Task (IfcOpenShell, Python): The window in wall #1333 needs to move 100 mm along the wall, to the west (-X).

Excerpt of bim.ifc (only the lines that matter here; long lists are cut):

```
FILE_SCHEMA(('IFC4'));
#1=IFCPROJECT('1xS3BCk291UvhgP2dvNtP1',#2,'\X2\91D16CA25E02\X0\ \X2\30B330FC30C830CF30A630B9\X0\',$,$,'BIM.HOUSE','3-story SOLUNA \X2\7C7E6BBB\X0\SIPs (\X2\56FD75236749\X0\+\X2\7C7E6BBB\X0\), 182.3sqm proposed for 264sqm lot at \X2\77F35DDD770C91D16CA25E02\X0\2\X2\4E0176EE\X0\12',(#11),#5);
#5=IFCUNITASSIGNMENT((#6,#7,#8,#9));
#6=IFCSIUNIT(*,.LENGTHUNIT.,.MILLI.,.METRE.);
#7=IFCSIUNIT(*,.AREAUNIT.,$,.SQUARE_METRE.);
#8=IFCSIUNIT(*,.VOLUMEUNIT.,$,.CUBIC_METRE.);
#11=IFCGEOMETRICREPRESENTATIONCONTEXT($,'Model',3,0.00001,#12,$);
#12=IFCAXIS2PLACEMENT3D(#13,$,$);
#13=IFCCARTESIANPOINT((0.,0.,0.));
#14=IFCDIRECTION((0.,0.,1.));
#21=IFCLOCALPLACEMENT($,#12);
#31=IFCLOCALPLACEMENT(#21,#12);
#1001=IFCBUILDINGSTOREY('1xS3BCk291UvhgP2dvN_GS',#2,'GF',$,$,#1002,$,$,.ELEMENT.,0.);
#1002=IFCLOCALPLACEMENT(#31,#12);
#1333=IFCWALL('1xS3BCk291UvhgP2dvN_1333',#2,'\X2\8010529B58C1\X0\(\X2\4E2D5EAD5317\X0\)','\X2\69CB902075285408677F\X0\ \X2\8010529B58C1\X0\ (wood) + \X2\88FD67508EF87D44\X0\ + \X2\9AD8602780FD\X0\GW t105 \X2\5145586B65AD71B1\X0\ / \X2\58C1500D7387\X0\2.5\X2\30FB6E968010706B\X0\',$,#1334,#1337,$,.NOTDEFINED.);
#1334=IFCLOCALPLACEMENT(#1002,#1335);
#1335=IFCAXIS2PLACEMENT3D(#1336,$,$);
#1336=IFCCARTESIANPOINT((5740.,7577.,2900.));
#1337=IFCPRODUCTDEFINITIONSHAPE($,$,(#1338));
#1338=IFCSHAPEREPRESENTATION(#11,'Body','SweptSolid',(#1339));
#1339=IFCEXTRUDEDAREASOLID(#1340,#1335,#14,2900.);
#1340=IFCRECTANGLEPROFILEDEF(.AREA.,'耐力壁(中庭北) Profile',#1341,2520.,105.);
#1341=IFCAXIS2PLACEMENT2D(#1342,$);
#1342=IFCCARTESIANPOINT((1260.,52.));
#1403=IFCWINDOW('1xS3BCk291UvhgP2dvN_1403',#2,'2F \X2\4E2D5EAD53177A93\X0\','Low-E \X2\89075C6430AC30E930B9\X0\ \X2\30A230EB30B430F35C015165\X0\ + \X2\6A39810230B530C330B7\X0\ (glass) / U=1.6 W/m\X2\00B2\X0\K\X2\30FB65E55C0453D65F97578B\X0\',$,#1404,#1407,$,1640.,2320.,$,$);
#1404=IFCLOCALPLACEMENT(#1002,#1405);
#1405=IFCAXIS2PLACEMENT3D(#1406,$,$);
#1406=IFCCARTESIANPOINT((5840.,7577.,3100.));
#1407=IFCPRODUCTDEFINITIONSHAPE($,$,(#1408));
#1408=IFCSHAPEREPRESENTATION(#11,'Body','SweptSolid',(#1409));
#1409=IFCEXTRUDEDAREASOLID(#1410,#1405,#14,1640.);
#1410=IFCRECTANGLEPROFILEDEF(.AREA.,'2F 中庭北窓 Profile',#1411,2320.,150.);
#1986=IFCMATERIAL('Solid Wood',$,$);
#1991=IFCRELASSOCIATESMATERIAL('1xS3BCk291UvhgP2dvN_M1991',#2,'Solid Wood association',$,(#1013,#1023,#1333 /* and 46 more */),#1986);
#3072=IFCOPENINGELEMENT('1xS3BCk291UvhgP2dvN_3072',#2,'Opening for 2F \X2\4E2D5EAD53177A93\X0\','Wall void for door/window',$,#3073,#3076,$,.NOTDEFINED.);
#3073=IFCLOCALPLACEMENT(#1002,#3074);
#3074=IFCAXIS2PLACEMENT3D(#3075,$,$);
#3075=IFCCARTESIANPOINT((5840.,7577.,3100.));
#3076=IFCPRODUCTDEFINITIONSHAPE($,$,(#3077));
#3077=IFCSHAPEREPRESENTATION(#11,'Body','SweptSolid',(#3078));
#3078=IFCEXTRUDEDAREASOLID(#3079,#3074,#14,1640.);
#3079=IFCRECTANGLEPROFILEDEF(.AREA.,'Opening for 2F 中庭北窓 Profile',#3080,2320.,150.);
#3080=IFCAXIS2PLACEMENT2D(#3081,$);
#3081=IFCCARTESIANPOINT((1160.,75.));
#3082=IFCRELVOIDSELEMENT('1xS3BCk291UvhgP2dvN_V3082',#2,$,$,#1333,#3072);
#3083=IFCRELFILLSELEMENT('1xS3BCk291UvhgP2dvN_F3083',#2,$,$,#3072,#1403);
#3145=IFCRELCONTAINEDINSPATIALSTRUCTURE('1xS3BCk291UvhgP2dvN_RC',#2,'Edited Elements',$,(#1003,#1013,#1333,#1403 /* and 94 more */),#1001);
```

```python
import ifcopenshell
import ifcopenshell.api.geometry
import ifcopenshell.util.placement
import ifcopenshell.util.unit

model = ifcopenshell.open("bim.ifc")
unit_scale = ifcopenshell.util.unit.calculate_unit_scale(model)

window = model.by_guid("1xS3BCk291UvhgP2dvN_1403")
opening = window.FillsVoids[0].RelatingOpeningElement
wall = opening.VoidsElements[0].RelatingBuildingElement

wall_matrix = ifcopenshell.util.placement.get_local_placement(wall.ObjectPlacement)
shift = wall_matrix[:3, 0] * -0.1 / unit_scale
before = ifcopenshell.util.placement.get_local_placement(window.ObjectPlacement)[:3, 3].copy()

# The window is not placed relative to its opening, so move both.
for product in (opening, window):
    matrix = ifcopenshell.util.placement.get_local_placement(product.ObjectPlacement)
    matrix[:3, 3] += shift
    ifcopenshell.api.geometry.edit_object_placement(model, product=product, matrix=matrix, is_si=False)

after = ifcopenshell.util.placement.get_local_placement(window.ObjectPlacement)[:3, 3]
print("window moved by", (after - before).round(3) + 0.0)

model.write("bim_edited.ifc")
```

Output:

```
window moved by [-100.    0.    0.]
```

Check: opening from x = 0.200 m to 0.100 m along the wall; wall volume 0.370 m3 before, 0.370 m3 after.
